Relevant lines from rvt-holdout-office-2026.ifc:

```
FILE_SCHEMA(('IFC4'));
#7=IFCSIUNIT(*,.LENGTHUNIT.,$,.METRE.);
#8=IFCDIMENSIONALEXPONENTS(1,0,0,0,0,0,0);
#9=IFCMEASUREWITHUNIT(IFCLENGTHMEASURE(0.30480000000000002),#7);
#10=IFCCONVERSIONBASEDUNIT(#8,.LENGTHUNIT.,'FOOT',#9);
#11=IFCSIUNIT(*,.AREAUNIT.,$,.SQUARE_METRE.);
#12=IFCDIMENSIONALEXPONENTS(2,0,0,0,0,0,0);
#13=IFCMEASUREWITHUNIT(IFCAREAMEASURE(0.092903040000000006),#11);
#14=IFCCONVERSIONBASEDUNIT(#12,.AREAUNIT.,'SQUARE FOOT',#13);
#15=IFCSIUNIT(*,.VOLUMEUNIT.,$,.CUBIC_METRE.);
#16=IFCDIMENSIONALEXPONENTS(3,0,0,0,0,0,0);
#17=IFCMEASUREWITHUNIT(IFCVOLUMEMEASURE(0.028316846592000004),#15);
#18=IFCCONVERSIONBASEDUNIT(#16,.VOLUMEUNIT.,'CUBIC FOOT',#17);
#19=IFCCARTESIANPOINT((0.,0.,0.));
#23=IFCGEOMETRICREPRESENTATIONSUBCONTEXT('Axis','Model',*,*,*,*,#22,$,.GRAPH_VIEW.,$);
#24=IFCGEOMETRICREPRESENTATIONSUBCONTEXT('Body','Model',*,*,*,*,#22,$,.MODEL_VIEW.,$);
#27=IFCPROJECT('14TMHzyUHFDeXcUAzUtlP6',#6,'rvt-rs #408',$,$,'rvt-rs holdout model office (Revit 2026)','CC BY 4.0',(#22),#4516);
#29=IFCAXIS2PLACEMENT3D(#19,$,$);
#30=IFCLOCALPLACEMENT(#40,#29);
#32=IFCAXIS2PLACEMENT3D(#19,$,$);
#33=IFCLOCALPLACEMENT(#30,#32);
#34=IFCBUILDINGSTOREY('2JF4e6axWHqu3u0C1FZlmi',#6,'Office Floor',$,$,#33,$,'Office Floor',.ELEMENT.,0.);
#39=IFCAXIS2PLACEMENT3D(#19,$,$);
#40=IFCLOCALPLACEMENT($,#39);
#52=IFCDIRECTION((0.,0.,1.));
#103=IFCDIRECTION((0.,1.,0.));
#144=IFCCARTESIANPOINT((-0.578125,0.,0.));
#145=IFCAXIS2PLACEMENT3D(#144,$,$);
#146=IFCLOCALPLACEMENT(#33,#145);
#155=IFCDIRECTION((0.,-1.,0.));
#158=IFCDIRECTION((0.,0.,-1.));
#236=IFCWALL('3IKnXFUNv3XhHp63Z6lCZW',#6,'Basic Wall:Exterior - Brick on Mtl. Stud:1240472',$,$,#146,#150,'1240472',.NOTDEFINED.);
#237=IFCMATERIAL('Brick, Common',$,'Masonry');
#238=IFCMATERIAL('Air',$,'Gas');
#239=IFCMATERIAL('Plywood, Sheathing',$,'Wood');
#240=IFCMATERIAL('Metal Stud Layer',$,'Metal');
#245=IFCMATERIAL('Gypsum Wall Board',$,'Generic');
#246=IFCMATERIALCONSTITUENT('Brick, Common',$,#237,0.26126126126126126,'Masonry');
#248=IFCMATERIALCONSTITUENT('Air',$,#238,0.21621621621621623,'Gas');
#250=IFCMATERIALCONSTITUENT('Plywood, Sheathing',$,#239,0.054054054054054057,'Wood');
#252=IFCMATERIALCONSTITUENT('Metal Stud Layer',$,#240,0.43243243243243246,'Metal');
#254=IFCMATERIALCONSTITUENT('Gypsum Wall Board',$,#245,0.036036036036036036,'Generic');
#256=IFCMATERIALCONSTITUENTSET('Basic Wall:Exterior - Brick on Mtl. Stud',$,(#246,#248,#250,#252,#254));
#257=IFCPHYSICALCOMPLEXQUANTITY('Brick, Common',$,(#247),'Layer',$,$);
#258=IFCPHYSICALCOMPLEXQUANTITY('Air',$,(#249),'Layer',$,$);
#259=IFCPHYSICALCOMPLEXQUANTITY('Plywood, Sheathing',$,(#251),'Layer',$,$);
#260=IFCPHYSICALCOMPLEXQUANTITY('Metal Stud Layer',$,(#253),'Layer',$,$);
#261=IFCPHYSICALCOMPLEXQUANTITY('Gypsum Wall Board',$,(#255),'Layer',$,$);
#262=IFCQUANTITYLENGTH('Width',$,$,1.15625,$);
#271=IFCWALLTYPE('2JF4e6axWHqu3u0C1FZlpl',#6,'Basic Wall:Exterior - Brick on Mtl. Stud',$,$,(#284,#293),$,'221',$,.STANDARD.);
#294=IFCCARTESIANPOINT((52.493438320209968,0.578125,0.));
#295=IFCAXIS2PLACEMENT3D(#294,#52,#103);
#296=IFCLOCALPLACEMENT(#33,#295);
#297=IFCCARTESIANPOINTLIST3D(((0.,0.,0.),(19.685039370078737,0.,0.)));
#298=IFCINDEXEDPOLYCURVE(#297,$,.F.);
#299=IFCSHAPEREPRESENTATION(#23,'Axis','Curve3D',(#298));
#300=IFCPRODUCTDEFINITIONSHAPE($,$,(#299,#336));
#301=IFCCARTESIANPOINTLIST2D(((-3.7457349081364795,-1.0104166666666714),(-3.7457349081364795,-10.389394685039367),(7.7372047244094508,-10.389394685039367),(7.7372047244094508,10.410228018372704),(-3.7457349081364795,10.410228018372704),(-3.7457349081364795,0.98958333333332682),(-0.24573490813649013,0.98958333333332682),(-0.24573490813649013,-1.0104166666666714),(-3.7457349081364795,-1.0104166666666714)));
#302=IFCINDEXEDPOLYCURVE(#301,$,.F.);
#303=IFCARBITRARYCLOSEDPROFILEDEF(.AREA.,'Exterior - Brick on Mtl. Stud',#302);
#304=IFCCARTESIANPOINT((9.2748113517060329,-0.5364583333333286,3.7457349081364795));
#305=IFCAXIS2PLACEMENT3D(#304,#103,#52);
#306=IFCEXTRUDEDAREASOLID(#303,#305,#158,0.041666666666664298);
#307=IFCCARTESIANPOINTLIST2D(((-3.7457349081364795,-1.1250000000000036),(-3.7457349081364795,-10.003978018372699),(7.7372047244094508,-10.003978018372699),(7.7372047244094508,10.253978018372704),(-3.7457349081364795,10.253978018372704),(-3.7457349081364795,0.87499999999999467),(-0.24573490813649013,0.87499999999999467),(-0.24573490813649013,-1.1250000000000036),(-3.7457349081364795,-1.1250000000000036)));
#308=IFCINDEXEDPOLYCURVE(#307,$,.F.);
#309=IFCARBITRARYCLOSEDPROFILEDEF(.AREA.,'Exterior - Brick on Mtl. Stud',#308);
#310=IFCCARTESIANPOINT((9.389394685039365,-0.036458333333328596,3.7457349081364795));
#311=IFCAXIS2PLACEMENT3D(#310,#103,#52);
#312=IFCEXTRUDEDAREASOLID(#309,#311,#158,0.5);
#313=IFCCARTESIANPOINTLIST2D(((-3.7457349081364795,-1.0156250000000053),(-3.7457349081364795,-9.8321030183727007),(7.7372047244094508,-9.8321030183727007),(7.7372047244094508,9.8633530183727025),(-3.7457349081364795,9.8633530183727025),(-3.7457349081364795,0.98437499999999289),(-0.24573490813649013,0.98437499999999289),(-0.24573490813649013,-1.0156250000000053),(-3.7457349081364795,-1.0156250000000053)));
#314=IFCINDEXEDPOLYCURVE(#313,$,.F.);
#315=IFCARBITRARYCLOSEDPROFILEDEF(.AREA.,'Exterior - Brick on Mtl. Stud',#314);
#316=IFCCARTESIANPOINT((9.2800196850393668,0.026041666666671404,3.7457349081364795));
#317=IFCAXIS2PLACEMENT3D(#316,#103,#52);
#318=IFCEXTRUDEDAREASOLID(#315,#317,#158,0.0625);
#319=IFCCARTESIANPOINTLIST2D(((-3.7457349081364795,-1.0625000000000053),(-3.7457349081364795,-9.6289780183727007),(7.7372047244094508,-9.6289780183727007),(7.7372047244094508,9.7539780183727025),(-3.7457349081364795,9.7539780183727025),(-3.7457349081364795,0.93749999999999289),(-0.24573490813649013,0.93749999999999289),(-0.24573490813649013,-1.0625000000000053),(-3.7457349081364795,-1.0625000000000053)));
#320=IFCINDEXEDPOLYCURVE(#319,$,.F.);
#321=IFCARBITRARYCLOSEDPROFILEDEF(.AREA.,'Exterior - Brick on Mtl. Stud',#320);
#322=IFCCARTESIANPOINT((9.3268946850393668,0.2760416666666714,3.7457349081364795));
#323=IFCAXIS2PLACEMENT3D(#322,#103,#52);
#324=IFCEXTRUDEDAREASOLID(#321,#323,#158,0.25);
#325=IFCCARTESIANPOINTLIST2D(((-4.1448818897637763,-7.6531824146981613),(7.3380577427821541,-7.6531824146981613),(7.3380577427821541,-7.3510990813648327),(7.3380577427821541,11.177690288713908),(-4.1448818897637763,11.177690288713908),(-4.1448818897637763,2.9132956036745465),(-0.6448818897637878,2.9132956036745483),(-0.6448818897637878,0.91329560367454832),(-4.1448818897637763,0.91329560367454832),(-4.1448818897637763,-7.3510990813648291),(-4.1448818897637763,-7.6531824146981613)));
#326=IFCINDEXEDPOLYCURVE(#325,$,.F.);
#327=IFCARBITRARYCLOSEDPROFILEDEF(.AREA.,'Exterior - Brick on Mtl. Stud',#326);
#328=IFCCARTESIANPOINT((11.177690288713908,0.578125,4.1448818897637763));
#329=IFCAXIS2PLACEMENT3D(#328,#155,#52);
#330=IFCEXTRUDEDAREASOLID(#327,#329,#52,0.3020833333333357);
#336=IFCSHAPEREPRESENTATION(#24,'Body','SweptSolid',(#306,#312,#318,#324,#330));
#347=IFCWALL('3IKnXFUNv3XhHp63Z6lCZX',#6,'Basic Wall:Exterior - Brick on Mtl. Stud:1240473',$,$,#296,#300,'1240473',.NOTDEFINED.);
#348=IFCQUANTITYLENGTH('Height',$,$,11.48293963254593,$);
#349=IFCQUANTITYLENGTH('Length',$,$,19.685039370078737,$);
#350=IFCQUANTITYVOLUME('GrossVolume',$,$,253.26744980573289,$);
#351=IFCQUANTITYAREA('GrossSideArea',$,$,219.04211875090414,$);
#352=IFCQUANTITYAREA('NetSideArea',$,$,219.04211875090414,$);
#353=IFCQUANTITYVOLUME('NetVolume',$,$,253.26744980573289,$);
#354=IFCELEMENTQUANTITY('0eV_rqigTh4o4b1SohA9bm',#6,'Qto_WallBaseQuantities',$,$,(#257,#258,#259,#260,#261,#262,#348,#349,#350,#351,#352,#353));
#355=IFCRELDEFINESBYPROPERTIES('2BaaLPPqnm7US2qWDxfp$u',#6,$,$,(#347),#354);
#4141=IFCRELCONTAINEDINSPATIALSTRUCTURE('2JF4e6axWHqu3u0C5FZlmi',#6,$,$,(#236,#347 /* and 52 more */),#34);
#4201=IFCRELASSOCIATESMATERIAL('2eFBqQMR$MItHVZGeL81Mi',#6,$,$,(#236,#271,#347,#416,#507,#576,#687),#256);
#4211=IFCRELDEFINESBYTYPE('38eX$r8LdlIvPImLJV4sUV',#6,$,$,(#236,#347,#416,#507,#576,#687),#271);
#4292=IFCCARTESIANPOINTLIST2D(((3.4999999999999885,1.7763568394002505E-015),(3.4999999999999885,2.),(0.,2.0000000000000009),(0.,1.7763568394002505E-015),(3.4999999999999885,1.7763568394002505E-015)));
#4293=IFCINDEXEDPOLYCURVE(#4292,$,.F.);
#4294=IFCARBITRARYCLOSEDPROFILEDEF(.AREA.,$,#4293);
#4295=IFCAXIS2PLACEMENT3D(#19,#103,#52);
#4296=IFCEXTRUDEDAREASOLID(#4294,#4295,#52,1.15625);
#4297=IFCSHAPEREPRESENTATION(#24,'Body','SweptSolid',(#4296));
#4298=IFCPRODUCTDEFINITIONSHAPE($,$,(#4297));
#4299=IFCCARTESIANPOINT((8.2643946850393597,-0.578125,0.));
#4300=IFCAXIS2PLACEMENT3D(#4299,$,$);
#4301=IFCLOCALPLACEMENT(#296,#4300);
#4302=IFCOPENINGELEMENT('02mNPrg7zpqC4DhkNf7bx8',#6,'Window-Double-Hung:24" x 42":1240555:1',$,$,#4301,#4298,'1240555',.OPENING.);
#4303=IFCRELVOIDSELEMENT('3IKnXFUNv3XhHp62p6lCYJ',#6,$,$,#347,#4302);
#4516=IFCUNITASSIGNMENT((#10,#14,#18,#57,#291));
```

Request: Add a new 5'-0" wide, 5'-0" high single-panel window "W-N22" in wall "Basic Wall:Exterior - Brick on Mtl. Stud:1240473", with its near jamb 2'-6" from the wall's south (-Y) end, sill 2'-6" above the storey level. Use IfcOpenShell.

```python
import numpy as np
import ifcopenshell
import ifcopenshell.api.feature
import ifcopenshell.api.geometry
import ifcopenshell.api.pset
import ifcopenshell.api.root
import ifcopenshell.api.spatial
import ifcopenshell.geom
import ifcopenshell.util.element
import ifcopenshell.util.placement
import ifcopenshell.util.representation
import ifcopenshell.util.shape
import ifcopenshell.util.unit

model = ifcopenshell.open("rvt-holdout-office-2026.ifc")
unit_scale = ifcopenshell.util.unit.calculate_unit_scale(model)
area_scale = ifcopenshell.util.unit.calculate_unit_scale(model, "AREAUNIT")
volume_scale = ifcopenshell.util.unit.calculate_unit_scale(model, "VOLUMEUNIT")
settings = ifcopenshell.geom.settings()


def volume(element):
    """Net volume in cubic metres, openings subtracted."""
    shape = ifcopenshell.geom.create_shape(settings, element)
    return ifcopenshell.util.shape.get_volume(shape.geometry)


wall = model.by_guid("3IKnXFUNv3XhHp63Z6lCZX")
storey = ifcopenshell.util.element.get_container(wall, ifc_class="IfcBuildingStorey")
context = ifcopenshell.util.representation.get_context(model, "Model", "Body", "MODEL_VIEW")
before = volume(wall)

width, height, from_end, sill = 1.524, 1.524, 0.762, 0.762  # metres

# The wall runs along its own X axis, and the end named is its -X end.
wall_shape = ifcopenshell.geom.create_shape(settings, wall)
x, y, z = ifcopenshell.util.shape.get_vertices(wall_shape.geometry).T
start = x.min() + from_end
face, thickness = float(y.min()), float(y.max() - y.min())
wall_matrix = ifcopenshell.util.placement.get_local_placement(wall.ObjectPlacement)
level = ifcopenshell.util.placement.get_local_placement(storey.ObjectPlacement)[2, 3]


def in_wall(x, y):
    """Placement at x, y metres in the wall's axes, at sill height."""
    matrix = wall_matrix.copy()
    matrix[:, 3] = wall_matrix @ np.array([x / unit_scale, y / unit_scale, 0.0, 1.0])
    matrix[2, 3] = level + sill / unit_scale
    return matrix


# Opening: a box that overshoots both wall faces by 50 mm.
opening = ifcopenshell.api.root.create_entity(model, ifc_class="IfcOpeningElement", predefined_type="OPENING")
box = ifcopenshell.api.geometry.add_wall_representation(
    model, context=context, length=width, height=height, thickness=thickness + 0.1
)
ifcopenshell.api.geometry.assign_representation(model, product=opening, representation=box)
ifcopenshell.api.geometry.edit_object_placement(model, product=opening, matrix=in_wall(start, face - 0.05), is_si=False)
ifcopenshell.api.feature.add_feature(model, feature=opening, element=wall)

window = ifcopenshell.api.root.create_entity(model, ifc_class="IfcWindow", name="W-N22", predefined_type="WINDOW")
window.OverallWidth, window.OverallHeight = width / unit_scale, height / unit_scale
window.PartitioningType = "SINGLE_PANEL"
body = ifcopenshell.api.geometry.add_window_representation(
    model,
    context=context,
    overall_width=window.OverallWidth,
    overall_height=window.OverallHeight,
    partition_type="SINGLE_PANEL",
)
ifcopenshell.api.geometry.assign_representation(model, product=window, representation=body)
ifcopenshell.api.spatial.assign_container(model, products=[window], relating_structure=storey)
ifcopenshell.api.feature.add_filling(model, opening=opening, element=window)

# Centre the window in the wall's thickness.
ifcopenshell.api.geometry.edit_object_placement(model, product=window, matrix=in_wall(start, face), is_si=False)
window_shape = ifcopenshell.geom.create_shape(settings, window)
depth = ifcopenshell.util.shape.get_vertices(window_shape.geometry)[:, 1]
offset = face + thickness / 2 - (depth.min() + depth.max()) / 2
ifcopenshell.api.geometry.edit_object_placement(model, product=window, matrix=in_wall(start, offset), is_si=False)

after = volume(wall)

# Update the wall's stored quantities.
qto = model.by_id(ifcopenshell.util.element.get_pset(wall, "Qto_WallBaseQuantities", should_inherit=False)["id"])
ifcopenshell.api.pset.edit_qto(model, qto=qto, properties={
    "NetSideArea": after / thickness / area_scale,
    "NetVolume": after / volume_scale,
})

print(f"wall volume {before:.3f} -> {after:.3f} m3")

model.write("rvt-holdout-office-2026_v2.ifc")
```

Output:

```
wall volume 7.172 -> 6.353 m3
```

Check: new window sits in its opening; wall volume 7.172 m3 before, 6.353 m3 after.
